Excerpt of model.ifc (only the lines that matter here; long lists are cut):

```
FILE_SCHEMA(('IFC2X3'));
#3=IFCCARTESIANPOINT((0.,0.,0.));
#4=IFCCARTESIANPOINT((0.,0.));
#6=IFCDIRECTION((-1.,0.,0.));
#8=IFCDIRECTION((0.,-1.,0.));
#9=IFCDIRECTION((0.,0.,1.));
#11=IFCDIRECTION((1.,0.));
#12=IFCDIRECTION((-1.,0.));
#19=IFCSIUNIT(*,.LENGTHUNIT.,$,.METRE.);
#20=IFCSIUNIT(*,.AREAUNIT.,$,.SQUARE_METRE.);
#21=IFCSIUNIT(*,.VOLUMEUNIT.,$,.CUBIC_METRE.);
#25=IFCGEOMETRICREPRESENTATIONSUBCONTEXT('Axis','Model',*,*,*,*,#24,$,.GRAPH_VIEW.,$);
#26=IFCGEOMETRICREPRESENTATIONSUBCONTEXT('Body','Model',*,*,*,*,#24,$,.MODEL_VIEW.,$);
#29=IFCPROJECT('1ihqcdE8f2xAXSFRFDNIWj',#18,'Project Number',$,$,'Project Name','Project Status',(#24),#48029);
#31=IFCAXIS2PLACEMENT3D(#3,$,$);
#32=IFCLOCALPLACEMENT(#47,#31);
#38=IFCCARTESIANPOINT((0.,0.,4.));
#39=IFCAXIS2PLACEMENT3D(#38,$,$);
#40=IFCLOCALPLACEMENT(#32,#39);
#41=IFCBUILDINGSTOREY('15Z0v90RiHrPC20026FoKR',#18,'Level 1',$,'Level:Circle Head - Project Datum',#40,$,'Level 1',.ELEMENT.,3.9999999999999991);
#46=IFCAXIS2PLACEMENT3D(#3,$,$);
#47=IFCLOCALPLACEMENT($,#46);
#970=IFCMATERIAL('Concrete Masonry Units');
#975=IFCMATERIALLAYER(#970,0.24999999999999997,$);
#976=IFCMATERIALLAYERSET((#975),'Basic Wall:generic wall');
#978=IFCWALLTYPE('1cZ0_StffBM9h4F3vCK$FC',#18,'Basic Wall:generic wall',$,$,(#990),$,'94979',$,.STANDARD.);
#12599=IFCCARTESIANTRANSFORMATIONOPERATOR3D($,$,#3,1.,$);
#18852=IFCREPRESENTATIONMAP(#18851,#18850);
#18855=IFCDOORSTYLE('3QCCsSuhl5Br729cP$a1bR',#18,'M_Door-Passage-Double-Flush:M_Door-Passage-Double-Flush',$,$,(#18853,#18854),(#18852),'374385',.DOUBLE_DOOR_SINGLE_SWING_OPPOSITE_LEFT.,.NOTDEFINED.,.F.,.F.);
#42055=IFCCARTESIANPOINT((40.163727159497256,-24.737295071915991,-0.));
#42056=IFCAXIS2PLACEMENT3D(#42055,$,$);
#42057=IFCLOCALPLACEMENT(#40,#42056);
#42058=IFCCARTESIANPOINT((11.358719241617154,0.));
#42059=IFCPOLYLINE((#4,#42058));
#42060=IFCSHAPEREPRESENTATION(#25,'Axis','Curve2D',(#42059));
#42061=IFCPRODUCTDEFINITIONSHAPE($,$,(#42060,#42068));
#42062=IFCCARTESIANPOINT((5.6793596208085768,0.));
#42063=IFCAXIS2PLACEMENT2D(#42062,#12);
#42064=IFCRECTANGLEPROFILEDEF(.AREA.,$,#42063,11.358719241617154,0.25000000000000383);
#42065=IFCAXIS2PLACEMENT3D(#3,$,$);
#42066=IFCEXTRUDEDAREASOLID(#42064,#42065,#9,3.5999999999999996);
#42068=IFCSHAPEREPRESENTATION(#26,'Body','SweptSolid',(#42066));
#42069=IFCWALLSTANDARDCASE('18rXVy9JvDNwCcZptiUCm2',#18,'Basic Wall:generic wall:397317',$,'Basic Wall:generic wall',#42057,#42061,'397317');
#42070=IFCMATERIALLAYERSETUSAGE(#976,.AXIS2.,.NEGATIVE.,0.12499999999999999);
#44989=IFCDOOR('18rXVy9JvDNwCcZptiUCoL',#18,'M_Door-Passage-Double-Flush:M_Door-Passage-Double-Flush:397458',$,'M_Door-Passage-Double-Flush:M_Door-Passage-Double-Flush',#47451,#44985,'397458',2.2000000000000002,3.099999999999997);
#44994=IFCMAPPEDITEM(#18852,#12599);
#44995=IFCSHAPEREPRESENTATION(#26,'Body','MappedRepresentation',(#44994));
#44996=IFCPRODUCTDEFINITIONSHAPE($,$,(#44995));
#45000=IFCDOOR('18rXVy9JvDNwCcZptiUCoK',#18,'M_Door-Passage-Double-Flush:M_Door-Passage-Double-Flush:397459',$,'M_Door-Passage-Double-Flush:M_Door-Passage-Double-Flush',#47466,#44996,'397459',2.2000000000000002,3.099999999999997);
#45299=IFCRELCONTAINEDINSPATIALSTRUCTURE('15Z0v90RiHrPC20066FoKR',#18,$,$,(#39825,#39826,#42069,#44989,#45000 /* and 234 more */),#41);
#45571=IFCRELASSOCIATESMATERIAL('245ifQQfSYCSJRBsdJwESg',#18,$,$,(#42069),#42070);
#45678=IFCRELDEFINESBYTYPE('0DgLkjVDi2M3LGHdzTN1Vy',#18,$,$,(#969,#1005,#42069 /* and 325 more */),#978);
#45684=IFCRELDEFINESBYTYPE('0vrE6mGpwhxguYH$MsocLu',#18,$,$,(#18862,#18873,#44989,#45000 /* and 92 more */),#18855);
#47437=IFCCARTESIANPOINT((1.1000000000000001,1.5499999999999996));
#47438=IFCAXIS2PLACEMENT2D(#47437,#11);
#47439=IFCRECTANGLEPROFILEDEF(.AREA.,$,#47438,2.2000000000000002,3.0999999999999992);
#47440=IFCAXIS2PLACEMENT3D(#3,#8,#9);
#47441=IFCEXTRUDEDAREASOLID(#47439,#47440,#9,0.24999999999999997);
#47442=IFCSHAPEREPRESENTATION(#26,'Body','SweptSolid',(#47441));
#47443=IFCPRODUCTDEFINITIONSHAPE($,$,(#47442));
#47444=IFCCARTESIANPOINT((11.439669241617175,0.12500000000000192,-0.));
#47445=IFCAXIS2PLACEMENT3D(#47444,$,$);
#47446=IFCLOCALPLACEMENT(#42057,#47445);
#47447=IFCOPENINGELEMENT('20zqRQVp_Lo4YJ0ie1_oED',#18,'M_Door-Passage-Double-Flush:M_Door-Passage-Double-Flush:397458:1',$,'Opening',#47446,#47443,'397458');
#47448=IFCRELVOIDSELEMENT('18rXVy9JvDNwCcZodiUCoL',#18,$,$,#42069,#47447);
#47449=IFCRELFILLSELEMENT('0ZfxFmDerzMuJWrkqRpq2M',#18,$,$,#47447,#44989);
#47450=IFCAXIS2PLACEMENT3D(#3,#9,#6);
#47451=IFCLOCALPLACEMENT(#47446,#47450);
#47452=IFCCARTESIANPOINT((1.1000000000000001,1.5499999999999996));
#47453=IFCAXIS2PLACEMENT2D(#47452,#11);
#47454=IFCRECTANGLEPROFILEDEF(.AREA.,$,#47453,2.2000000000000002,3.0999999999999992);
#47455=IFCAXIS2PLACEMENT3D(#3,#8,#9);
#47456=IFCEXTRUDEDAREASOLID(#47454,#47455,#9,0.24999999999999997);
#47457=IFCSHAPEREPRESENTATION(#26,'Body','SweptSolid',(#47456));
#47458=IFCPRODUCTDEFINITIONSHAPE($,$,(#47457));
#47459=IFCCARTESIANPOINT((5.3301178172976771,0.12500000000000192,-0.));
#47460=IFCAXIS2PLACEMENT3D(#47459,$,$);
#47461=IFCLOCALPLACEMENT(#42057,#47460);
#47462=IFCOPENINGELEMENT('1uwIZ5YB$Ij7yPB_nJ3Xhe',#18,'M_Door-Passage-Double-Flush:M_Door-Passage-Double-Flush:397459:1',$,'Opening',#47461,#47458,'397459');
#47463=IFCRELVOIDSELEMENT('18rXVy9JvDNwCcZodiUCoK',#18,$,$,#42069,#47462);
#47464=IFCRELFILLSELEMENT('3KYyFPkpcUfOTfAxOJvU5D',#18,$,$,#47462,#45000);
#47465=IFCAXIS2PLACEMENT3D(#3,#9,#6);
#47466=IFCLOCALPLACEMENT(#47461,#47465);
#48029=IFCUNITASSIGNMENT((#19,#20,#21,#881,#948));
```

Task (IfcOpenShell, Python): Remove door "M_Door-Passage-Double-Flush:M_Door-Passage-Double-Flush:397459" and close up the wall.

```python
import ifcopenshell
import ifcopenshell.api.feature
import ifcopenshell.api.root
import ifcopenshell.geom
import ifcopenshell.util.shape

model = ifcopenshell.open("model.ifc")
settings = ifcopenshell.geom.settings()


def volume(element):
    """Net volume in cubic metres, openings subtracted."""
    shape = ifcopenshell.geom.create_shape(settings, element)
    return ifcopenshell.util.shape.get_volume(shape.geometry)


door = model.by_guid("18rXVy9JvDNwCcZptiUCoK")
opening = door.FillsVoids[0].RelatingOpeningElement
wall = opening.VoidsElements[0].RelatingBuildingElement
before = volume(wall)

ifcopenshell.api.root.remove_product(model, product=door)
ifcopenshell.api.feature.remove_feature(model, feature=opening)

after = volume(wall)

print(f"wall volume {before:.3f} -> {after:.3f} m3")

model.write("model_edited.ifc")
```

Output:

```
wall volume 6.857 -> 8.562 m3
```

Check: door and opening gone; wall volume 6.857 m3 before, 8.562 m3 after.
